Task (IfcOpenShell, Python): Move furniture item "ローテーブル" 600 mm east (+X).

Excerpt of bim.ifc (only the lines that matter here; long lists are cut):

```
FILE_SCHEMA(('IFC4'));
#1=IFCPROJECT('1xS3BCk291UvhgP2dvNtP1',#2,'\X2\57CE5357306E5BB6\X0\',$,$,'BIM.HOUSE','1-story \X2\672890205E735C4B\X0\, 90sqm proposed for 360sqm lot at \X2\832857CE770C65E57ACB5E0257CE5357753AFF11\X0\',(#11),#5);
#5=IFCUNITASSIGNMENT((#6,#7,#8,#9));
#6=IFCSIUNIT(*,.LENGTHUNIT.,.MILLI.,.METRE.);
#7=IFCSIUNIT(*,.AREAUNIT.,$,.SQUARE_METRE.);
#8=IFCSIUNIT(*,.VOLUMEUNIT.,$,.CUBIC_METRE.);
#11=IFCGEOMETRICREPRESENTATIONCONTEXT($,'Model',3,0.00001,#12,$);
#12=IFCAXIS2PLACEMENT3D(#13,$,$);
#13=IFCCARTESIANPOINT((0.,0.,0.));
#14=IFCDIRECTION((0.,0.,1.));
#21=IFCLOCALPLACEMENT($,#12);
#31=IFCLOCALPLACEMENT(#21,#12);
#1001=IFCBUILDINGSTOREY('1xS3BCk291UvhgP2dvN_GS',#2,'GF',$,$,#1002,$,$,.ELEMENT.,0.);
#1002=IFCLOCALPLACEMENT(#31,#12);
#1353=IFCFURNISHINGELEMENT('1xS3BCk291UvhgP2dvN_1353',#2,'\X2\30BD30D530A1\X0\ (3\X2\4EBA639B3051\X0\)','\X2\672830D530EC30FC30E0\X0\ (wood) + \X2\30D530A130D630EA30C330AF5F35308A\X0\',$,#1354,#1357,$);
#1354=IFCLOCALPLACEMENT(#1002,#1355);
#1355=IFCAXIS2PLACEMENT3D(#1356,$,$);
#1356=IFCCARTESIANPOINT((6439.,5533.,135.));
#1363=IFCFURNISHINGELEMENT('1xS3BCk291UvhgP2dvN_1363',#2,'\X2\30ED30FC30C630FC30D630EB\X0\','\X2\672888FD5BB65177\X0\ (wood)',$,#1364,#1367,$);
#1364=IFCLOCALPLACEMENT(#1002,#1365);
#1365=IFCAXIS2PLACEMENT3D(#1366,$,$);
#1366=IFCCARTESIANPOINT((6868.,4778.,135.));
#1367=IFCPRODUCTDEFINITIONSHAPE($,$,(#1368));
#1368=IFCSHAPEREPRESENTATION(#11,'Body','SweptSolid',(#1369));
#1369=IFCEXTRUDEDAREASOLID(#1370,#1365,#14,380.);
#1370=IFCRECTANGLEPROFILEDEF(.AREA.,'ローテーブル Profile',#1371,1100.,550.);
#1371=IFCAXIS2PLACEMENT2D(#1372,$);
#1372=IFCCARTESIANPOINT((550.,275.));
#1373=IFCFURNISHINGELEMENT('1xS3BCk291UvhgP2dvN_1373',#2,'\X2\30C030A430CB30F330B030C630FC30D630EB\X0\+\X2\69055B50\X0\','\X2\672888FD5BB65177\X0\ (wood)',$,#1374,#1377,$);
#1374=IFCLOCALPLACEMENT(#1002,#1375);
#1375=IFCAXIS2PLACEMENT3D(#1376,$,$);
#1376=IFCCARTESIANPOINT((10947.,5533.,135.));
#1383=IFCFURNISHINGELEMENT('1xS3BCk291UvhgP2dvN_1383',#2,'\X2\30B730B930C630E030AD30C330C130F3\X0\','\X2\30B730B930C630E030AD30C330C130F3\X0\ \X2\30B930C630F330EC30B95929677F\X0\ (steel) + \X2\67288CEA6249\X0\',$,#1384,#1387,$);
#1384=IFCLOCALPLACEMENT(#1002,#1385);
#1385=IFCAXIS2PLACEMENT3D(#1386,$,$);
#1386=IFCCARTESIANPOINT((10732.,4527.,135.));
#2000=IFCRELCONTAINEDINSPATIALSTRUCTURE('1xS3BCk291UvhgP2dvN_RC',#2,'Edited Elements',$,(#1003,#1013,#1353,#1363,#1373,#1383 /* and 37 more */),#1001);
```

```python
import ifcopenshell
import ifcopenshell.api.geometry
import ifcopenshell.util.placement
import ifcopenshell.util.unit

model = ifcopenshell.open("bim.ifc")
unit_scale = ifcopenshell.util.unit.calculate_unit_scale(model)

item = model.by_guid("1xS3BCk291UvhgP2dvN_1363")
matrix = ifcopenshell.util.placement.get_local_placement(item.ObjectPlacement)
matrix[0, 3] += 0.6 / unit_scale
ifcopenshell.api.geometry.edit_object_placement(model, product=item, matrix=matrix, is_si=False)

print(ifcopenshell.util.placement.get_local_placement(item.ObjectPlacement).round(3) + 0.0)

model.write("bim-out.ifc")
```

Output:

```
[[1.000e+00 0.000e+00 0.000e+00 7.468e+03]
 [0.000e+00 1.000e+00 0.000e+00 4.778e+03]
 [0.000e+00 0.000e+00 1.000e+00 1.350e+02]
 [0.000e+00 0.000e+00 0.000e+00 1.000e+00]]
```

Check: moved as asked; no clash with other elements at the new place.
